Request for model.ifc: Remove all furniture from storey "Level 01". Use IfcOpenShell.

First a look at what the model holds.

```python
import ifcopenshell
import ifcopenshell.util.element

model = ifcopenshell.open("model.ifc")
print(model.schema)
storey = next(s for s in model.by_type("IfcBuildingStorey") if s.Name == "Level 01")
furniture = [e for e in ifcopenshell.util.element.get_decomposition(storey) if e.is_a("IfcFurnishingElement")]
seen = {}
for e in furniture:
    element_type = ifcopenshell.util.element.get_type(e)
    name = element_type.Name if element_type not in (None, e) else None
    seen[name] = seen.get(name, 0) + 1
for name, count in sorted(seen.items(), key=str):
    print(count, "x", name)
```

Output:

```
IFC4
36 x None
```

```python
import ifcopenshell
import ifcopenshell.api.root
import ifcopenshell.util.element

model = ifcopenshell.open("model.ifc")

storey = next(s for s in model.by_type("IfcBuildingStorey") if s.Name == "Level 01")
furniture = [e for e in ifcopenshell.util.element.get_decomposition(storey) if e.is_a("IfcFurnishingElement")]

for e in furniture:
    ifcopenshell.api.root.remove_product(model, product=e)
print(len(furniture), "removed")

model.write("model_v2.ifc")
```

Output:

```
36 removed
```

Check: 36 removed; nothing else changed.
